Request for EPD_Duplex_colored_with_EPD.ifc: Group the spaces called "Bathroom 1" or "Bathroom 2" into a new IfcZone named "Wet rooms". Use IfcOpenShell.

First a look at what the model holds.

```python
import ifcopenshell

model = ifcopenshell.open("EPD_Duplex_colored_with_EPD.ifc")
print(model.schema)
seen = {}
for space in model.by_type("IfcSpace"):
    seen[space.LongName] = seen.get(space.LongName, 0) + 1
for name, count in sorted(seen.items(), key=str):
    print(count, "x", name)
print("zones:", [z.Name for z in model.by_type("IfcZone")][:20])
```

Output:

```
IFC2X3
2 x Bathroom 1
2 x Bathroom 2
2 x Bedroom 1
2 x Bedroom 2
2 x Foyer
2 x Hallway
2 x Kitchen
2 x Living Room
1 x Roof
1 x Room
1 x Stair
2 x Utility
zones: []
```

```python
import ifcopenshell
import ifcopenshell.api.group
import ifcopenshell.api.root

model = ifcopenshell.open("EPD_Duplex_colored_with_EPD.ifc")

names = {"Bathroom 1", "Bathroom 2"}
spaces = [s for s in model.by_type("IfcSpace") if s.LongName in names]

zone = ifcopenshell.api.root.create_entity(model, ifc_class="IfcZone", name="Wet rooms")
ifcopenshell.api.group.assign_group(model, products=spaces, group=zone)
print(len(spaces), "spaces in", zone.Name)

model.write("EPD_Duplex_colored_with_EPD-out.ifc")
```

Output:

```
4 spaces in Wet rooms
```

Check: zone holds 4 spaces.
